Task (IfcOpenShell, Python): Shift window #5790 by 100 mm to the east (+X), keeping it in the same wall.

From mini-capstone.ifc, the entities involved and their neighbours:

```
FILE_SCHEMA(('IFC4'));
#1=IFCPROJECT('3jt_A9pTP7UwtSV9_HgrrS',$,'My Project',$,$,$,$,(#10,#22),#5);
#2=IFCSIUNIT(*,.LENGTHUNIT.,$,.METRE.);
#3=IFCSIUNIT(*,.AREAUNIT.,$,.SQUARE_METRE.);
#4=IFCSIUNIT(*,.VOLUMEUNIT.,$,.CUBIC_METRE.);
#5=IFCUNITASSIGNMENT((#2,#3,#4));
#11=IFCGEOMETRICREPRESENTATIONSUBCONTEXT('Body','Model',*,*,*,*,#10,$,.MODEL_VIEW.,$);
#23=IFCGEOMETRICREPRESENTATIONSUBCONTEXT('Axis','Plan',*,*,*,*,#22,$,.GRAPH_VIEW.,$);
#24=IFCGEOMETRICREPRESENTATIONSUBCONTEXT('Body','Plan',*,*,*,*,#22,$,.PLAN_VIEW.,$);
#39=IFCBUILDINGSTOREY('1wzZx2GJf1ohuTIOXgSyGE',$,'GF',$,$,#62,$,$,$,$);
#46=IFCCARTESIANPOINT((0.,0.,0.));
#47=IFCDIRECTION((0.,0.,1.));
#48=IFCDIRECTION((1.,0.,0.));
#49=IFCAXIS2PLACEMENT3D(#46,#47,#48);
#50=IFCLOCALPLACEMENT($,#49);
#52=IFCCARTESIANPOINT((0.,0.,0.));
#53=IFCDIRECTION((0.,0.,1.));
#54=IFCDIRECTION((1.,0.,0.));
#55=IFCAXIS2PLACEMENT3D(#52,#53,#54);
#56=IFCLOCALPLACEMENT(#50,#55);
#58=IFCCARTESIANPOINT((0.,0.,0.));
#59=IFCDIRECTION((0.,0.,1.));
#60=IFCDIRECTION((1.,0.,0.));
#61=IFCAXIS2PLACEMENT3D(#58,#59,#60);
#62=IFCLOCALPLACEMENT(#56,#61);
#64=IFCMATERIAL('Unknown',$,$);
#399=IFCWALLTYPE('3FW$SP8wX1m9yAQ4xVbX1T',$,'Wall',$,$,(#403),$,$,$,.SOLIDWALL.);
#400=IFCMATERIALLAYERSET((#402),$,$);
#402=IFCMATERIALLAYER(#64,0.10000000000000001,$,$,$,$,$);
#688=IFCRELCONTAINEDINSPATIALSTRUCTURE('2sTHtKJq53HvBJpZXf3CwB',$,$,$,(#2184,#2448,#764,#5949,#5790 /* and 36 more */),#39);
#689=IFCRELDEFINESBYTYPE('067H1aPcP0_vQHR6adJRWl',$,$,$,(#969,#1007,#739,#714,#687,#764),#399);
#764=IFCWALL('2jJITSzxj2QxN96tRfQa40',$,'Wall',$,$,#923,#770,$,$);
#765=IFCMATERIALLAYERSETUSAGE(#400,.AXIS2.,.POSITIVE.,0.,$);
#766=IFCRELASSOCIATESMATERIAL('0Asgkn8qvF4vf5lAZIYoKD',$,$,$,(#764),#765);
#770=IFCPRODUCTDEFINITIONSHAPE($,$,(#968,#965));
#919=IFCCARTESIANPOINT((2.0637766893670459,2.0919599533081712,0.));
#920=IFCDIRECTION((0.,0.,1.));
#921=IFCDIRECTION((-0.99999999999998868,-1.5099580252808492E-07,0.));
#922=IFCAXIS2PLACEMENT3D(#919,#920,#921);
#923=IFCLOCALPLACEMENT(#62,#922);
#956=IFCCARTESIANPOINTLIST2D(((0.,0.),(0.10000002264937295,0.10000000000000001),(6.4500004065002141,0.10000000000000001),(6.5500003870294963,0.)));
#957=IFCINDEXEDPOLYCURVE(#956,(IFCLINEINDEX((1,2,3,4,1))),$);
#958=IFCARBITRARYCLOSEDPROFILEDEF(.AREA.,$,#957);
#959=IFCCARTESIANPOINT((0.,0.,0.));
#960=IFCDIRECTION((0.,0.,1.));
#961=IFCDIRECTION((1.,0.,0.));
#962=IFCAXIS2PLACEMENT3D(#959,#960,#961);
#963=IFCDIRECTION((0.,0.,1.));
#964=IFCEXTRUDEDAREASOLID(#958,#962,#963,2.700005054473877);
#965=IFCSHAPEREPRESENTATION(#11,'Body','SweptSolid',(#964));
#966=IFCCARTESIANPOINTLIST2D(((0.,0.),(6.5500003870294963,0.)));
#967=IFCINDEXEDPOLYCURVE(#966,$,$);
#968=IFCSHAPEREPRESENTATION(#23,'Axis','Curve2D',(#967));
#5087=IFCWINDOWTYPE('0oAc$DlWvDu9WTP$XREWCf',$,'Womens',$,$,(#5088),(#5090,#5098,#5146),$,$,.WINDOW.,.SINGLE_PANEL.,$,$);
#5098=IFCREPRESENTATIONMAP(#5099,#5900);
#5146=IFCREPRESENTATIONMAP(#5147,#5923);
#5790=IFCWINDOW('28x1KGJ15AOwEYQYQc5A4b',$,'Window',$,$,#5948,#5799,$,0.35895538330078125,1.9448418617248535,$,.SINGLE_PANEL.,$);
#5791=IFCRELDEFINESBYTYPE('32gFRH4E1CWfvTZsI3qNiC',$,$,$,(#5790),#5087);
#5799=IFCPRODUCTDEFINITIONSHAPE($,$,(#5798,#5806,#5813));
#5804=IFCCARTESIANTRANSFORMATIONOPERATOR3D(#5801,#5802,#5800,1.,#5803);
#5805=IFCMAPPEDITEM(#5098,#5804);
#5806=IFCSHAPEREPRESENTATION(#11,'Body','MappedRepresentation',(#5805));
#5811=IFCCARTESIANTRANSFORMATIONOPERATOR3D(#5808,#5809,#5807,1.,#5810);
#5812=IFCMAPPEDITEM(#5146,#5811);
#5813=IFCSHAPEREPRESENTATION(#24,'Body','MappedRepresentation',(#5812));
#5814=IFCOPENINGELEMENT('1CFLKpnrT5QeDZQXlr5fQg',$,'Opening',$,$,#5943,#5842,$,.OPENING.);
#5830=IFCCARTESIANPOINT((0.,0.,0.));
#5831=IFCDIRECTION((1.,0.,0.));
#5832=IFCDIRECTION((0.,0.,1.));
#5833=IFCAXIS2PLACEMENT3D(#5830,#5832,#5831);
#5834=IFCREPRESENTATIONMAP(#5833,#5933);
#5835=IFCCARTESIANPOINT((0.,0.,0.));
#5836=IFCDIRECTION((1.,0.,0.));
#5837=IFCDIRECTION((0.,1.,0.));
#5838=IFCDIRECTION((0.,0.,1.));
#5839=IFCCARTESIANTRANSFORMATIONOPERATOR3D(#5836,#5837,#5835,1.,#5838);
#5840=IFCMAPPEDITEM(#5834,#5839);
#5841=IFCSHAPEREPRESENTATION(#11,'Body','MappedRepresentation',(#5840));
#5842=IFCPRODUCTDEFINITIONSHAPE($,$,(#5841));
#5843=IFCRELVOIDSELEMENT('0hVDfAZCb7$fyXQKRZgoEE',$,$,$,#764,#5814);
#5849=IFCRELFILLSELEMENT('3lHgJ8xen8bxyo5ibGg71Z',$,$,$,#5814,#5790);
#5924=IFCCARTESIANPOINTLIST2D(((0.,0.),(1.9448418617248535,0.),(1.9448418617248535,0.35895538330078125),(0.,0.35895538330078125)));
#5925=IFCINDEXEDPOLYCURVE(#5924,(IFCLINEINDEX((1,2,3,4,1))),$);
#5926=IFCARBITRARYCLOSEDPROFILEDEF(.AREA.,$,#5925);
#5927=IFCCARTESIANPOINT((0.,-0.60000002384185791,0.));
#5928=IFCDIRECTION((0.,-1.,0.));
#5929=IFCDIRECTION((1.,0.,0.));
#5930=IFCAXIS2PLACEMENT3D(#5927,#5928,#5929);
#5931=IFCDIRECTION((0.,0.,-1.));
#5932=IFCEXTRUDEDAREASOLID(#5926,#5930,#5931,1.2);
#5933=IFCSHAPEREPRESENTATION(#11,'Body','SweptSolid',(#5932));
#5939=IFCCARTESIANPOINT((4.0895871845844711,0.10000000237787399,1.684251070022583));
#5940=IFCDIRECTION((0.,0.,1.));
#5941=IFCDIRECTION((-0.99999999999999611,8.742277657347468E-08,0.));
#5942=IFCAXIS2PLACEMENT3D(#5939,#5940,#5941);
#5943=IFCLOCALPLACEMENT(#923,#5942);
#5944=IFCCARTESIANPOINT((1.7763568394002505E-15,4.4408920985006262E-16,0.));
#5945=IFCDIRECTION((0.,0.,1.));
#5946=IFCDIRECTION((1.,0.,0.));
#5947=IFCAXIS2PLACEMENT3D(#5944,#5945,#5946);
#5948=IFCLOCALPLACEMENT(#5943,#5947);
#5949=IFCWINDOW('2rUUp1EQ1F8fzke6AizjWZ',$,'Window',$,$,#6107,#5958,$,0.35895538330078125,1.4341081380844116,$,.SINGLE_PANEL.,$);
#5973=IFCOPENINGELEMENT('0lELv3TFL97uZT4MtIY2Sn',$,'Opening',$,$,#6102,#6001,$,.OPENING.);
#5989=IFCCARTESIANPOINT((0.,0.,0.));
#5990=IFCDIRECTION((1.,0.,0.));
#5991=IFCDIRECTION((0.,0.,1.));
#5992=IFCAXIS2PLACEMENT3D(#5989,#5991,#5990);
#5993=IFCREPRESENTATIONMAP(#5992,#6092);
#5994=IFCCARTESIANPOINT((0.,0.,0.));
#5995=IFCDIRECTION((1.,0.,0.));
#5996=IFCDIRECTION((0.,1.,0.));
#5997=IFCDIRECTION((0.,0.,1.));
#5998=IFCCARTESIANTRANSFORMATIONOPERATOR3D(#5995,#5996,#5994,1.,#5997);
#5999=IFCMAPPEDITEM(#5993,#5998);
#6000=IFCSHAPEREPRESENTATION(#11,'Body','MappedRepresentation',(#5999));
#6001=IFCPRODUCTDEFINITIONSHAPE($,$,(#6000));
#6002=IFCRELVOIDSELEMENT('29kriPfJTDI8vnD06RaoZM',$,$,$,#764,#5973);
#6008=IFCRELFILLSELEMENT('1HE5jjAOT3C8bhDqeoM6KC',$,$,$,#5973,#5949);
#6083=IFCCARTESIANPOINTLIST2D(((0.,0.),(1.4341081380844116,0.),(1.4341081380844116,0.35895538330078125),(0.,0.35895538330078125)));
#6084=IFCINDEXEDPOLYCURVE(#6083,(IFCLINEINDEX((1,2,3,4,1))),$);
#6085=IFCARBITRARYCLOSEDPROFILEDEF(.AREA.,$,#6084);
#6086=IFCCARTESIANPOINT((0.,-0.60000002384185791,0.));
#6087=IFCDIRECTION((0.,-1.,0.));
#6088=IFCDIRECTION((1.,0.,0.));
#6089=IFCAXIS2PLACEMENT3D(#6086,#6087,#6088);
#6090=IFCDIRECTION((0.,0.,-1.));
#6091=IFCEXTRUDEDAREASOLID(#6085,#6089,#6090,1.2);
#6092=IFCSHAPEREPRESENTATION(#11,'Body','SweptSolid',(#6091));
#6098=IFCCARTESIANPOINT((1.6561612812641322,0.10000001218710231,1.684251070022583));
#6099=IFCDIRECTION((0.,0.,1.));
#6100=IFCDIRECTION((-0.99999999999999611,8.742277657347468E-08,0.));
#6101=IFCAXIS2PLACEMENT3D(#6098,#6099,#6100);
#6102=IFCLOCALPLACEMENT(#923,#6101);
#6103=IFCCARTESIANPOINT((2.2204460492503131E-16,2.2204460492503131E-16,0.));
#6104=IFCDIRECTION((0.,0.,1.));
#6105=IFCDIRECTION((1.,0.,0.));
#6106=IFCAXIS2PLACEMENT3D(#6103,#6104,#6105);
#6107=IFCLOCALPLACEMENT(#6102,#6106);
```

```python
import ifcopenshell
import ifcopenshell.api.geometry
import ifcopenshell.util.placement
import ifcopenshell.util.unit

model = ifcopenshell.open("mini-capstone.ifc")
unit_scale = ifcopenshell.util.unit.calculate_unit_scale(model)

window = model.by_id(5790)
opening = window.FillsVoids[0].RelatingOpeningElement
wall = opening.VoidsElements[0].RelatingBuildingElement

wall_matrix = ifcopenshell.util.placement.get_local_placement(wall.ObjectPlacement)
shift = wall_matrix[:3, 0] * -0.1 / unit_scale
before = ifcopenshell.util.placement.get_local_placement(window.ObjectPlacement)[:3, 3].copy()

# The window is placed relative to its opening, so it follows when the opening moves.
matrix = ifcopenshell.util.placement.get_local_placement(opening.ObjectPlacement)
matrix[:3, 3] += shift
ifcopenshell.api.geometry.edit_object_placement(
    model, product=opening, matrix=matrix, is_si=False, should_transform_children=True
)

after = ifcopenshell.util.placement.get_local_placement(window.ObjectPlacement)[:3, 3]
print("window moved by", (after - before).round(3) + 0.0)

model.write("mini-capstone_v2.ifc")
```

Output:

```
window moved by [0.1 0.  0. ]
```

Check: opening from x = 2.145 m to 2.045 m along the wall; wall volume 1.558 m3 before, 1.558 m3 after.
